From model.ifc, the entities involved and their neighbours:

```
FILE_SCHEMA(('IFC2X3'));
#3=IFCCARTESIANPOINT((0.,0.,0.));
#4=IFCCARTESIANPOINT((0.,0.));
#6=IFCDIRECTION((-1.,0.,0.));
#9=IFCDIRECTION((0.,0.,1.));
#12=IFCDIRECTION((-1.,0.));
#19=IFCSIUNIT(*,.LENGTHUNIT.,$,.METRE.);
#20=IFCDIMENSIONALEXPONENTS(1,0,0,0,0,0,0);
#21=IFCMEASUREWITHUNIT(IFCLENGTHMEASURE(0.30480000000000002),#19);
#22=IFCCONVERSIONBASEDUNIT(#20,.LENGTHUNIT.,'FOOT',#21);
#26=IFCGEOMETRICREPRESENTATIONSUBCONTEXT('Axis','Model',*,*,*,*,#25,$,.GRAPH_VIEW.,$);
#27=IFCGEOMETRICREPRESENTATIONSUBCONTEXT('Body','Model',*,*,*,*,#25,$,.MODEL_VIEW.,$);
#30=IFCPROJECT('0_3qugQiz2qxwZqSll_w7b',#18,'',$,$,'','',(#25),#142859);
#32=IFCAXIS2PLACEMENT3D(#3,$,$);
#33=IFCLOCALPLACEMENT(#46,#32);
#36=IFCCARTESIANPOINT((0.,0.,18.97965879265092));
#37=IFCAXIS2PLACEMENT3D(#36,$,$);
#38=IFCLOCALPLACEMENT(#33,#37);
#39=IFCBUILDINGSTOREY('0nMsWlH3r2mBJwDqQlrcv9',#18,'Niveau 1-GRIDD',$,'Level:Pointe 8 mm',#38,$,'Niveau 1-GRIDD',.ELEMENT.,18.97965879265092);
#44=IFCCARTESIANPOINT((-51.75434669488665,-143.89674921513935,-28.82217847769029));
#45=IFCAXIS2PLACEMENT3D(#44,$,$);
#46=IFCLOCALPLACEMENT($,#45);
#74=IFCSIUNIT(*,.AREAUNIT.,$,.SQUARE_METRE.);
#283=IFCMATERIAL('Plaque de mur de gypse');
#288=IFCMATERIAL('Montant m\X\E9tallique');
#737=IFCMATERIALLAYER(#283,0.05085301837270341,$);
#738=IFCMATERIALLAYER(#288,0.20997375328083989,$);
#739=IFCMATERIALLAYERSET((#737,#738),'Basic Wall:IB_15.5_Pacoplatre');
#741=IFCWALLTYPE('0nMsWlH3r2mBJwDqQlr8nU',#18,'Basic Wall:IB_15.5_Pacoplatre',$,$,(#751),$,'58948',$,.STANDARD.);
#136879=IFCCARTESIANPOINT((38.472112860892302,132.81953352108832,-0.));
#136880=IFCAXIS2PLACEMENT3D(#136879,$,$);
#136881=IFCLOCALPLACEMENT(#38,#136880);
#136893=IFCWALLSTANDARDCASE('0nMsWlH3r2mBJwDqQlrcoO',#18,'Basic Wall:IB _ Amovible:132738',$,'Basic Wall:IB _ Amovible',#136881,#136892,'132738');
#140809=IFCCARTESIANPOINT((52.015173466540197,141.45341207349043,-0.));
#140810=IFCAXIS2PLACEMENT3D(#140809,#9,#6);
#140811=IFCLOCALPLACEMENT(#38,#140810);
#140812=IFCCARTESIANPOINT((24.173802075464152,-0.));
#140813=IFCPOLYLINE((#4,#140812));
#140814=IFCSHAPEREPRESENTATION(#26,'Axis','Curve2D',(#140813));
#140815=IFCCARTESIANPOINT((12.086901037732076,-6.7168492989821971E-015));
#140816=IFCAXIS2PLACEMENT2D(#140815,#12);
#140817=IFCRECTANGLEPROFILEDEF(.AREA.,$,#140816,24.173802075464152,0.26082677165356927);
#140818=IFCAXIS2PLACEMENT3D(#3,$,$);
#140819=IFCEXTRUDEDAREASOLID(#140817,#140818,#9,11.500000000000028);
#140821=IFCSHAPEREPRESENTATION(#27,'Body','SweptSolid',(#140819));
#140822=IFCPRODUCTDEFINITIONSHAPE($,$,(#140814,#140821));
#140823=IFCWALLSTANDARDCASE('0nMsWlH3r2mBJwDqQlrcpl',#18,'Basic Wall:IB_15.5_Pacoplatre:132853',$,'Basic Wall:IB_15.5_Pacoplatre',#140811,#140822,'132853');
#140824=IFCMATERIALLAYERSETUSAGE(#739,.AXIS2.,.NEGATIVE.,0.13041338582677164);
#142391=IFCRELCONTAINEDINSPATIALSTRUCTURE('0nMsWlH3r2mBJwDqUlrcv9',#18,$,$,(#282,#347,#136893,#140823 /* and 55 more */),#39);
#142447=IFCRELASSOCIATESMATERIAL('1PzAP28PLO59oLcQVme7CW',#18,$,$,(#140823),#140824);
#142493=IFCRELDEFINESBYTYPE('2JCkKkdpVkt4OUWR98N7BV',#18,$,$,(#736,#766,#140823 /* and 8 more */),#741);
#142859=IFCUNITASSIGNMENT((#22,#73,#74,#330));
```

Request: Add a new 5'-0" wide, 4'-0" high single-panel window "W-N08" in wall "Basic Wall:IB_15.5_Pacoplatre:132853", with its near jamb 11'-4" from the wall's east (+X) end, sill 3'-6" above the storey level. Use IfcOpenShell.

```python
import numpy as np
import ifcopenshell
import ifcopenshell.api.feature
import ifcopenshell.api.geometry
import ifcopenshell.api.root
import ifcopenshell.api.spatial
import ifcopenshell.api.type
import ifcopenshell.geom
import ifcopenshell.util.element
import ifcopenshell.util.placement
import ifcopenshell.util.representation
import ifcopenshell.util.shape
import ifcopenshell.util.unit

model = ifcopenshell.open("model.ifc")
unit_scale = ifcopenshell.util.unit.calculate_unit_scale(model)
settings = ifcopenshell.geom.settings()


def volume(element):
    """Net volume in cubic metres, openings subtracted."""
    shape = ifcopenshell.geom.create_shape(settings, element)
    return ifcopenshell.util.shape.get_volume(shape.geometry)


wall = model.by_guid("0nMsWlH3r2mBJwDqQlrcpl")
storey = ifcopenshell.util.element.get_container(wall, ifc_class="IfcBuildingStorey")
context = ifcopenshell.util.representation.get_context(model, "Model", "Body", "MODEL_VIEW")
before = volume(wall)

width, height, from_end, sill = 1.524, 1.2192, 3.4544, 1.0668  # metres

# The wall runs along its own X axis, and the end named is its -X end.
wall_shape = ifcopenshell.geom.create_shape(settings, wall)
x, y, z = ifcopenshell.util.shape.get_vertices(wall_shape.geometry).T
start = x.min() + from_end
face, thickness = float(y.min()), float(y.max() - y.min())
wall_matrix = ifcopenshell.util.placement.get_local_placement(wall.ObjectPlacement)
level = ifcopenshell.util.placement.get_local_placement(storey.ObjectPlacement)[2, 3]


def in_wall(x, y):
    """Placement at x, y metres in the wall's axes, at sill height."""
    matrix = wall_matrix.copy()
    matrix[:, 3] = wall_matrix @ np.array([x / unit_scale, y / unit_scale, 0.0, 1.0])
    matrix[2, 3] = level + sill / unit_scale
    return matrix


# Opening: a box that overshoots both wall faces by 50 mm.
opening = ifcopenshell.api.root.create_entity(model, ifc_class="IfcOpeningElement")
box = ifcopenshell.api.geometry.add_wall_representation(
    model, context=context, length=width, height=height, thickness=thickness + 0.1
)
ifcopenshell.api.geometry.assign_representation(model, product=opening, representation=box)
ifcopenshell.api.geometry.edit_object_placement(model, product=opening, matrix=in_wall(start, face - 0.05), is_si=False)
ifcopenshell.api.feature.add_feature(model, feature=opening, element=wall)

window = ifcopenshell.api.root.create_entity(model, ifc_class="IfcWindow", name="W-N08")
window.OverallWidth, window.OverallHeight = width / unit_scale, height / unit_scale
body = ifcopenshell.api.geometry.add_window_representation(
    model,
    context=context,
    overall_width=window.OverallWidth,
    overall_height=window.OverallHeight,
    partition_type="SINGLE_PANEL",
)
ifcopenshell.api.geometry.assign_representation(model, product=window, representation=body)
ifcopenshell.api.spatial.assign_container(model, products=[window], relating_structure=storey)
fills = ifcopenshell.api.feature.add_filling(model, opening=opening, element=window)
fills.OwnerHistory = window.OwnerHistory  # required in IFC2X3

# IFC2X3 keeps the operation on the window style.
style = ifcopenshell.api.root.create_entity(model, ifc_class="IfcWindowStyle", name="W-N08")
style.OperationType, style.ConstructionType = "SINGLE_PANEL", "NOTDEFINED"
style.ParameterTakesPrecedence = style.Sizeable = False
ifcopenshell.api.type.assign_type(model, related_objects=[window], relating_type=style)

# Centre the window in the wall's thickness.
ifcopenshell.api.geometry.edit_object_placement(model, product=window, matrix=in_wall(start, face), is_si=False)
window_shape = ifcopenshell.geom.create_shape(settings, window)
depth = ifcopenshell.util.shape.get_vertices(window_shape.geometry)[:, 1]
offset = face + thickness / 2 - (depth.min() + depth.max()) / 2
ifcopenshell.api.geometry.edit_object_placement(model, product=window, matrix=in_wall(start, offset), is_si=False)

after = volume(wall)

print(f"wall volume {before:.3f} -> {after:.3f} m3")

model.write("model_rev.ifc")
```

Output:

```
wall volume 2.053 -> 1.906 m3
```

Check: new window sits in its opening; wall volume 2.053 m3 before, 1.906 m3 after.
